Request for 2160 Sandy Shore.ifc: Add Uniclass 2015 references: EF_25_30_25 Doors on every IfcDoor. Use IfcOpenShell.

First a look at what the model holds.

```python
import ifcopenshell

model = ifcopenshell.open("2160 Sandy Shore.ifc")
print(model.schema)
print("classifications:", [c.Name for c in model.by_type("IfcClassification")])
for ifc_class in ("IfcDoor", "IfcRoof", "IfcStair", "IfcWall", "IfcWindow"):
    print(ifc_class, len(model.by_type(ifc_class)))
```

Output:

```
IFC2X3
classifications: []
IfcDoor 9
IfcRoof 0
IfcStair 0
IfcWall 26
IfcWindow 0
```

```python
import ifcopenshell
import ifcopenshell.api.classification

model = ifcopenshell.open("2160 Sandy Shore.ifc")

# IFC2X3 requires Source and Edition and has no link from the project to the system.
system = model.create_entity("IfcClassification", Source="NBS", Edition="2015", Name="Uniclass 2015")

codes = {
    "IfcDoor": ("EF_25_30_25", "Doors"),
}
for ifc_class, (code, name) in codes.items():
    products = model.by_type(ifc_class)
    ifcopenshell.api.classification.add_reference(
        model, products=products, classification=system, identification=code, name=name
    )
    print(code, len(products))

model.write("2160 Sandy Shore_v2.ifc")
```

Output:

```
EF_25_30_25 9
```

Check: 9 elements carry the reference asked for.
